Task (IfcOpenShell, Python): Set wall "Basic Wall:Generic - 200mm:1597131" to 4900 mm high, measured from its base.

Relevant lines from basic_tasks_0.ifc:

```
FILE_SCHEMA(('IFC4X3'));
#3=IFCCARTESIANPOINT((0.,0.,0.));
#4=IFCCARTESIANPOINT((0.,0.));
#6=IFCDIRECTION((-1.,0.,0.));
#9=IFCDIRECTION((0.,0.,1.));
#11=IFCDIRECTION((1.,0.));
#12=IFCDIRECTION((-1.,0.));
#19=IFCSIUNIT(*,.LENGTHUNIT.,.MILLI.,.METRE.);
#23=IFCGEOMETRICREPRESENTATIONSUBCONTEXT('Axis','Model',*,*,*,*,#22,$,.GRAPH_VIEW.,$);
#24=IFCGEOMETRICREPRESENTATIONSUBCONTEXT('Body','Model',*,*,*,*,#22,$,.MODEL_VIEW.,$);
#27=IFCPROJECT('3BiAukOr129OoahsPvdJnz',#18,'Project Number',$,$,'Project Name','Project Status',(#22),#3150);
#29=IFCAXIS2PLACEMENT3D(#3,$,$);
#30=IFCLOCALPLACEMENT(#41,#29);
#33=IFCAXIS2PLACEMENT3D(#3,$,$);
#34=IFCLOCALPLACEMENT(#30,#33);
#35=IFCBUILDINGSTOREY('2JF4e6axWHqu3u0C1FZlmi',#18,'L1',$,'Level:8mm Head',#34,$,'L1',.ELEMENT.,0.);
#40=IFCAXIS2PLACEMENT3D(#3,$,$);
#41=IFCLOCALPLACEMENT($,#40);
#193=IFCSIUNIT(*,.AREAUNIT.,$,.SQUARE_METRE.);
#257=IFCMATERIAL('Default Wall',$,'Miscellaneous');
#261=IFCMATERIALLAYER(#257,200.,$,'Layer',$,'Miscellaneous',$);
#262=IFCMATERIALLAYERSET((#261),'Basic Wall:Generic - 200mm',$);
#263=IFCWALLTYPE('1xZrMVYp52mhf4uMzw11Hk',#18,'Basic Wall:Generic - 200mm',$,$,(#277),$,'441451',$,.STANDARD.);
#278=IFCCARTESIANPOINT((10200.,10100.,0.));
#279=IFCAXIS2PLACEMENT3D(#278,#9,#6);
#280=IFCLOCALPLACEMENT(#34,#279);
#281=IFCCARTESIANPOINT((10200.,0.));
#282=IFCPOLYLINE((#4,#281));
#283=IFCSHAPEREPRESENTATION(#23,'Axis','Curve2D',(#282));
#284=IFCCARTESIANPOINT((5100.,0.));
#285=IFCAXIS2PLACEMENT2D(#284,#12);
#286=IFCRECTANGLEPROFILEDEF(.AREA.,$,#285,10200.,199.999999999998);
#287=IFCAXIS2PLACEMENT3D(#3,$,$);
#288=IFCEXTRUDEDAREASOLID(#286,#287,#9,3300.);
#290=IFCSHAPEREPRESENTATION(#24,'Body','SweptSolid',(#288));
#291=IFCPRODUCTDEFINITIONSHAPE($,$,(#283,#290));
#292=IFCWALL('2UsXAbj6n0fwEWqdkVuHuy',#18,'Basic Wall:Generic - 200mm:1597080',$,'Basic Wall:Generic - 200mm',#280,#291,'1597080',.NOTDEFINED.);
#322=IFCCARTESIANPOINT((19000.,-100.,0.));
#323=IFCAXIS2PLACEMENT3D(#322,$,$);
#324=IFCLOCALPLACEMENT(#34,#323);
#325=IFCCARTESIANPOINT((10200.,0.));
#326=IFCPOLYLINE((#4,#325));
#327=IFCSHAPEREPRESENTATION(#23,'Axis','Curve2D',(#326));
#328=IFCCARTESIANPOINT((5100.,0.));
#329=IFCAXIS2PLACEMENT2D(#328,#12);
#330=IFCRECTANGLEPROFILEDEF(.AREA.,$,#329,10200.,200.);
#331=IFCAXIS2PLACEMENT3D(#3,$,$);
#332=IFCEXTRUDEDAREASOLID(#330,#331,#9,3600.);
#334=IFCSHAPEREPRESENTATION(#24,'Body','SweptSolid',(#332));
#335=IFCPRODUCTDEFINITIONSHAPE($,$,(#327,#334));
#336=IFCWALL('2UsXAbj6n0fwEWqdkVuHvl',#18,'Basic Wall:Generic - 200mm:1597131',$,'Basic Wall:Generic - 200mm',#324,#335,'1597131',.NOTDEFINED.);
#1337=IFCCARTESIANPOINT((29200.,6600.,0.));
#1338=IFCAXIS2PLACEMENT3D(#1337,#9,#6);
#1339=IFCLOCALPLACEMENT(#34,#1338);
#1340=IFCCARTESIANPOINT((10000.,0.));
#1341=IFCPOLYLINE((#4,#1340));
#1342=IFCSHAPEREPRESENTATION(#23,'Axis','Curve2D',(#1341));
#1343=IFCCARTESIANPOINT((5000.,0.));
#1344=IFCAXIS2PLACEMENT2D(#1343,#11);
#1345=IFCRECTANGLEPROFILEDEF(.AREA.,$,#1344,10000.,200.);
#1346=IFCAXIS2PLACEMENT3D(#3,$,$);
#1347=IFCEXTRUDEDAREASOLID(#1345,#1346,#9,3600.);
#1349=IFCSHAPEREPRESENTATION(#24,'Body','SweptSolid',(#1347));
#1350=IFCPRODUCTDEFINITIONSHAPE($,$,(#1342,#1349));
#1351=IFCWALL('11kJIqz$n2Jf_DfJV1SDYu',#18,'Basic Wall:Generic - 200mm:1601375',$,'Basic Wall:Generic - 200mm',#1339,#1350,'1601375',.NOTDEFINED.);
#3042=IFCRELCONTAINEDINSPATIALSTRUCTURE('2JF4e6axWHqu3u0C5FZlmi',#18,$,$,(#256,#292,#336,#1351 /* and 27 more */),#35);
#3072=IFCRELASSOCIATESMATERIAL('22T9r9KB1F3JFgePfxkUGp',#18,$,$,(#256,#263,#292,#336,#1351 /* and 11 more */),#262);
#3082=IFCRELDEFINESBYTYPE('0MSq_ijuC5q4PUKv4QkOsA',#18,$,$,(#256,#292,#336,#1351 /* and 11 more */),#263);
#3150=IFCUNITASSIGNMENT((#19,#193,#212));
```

```python
import ifcopenshell
import ifcopenshell.geom
import ifcopenshell.util.representation
import ifcopenshell.util.shape
import ifcopenshell.util.unit

model = ifcopenshell.open("basic_tasks_0.ifc")
unit_scale = ifcopenshell.util.unit.calculate_unit_scale(model)
settings = ifcopenshell.geom.settings()


def volume(element):
    """Net volume in cubic metres, openings subtracted."""
    shape = ifcopenshell.geom.create_shape(settings, element)
    return ifcopenshell.util.shape.get_volume(shape.geometry)


wall = model.by_guid("2UsXAbj6n0fwEWqdkVuHvl")
before = volume(wall)

body = ifcopenshell.util.representation.get_representation(wall, "Model", "Body")
solid = body.Items[0]
old_height = solid.Depth
solid.Depth = 4.9 / unit_scale
after = volume(wall)

print(f"height {old_height:g} -> {solid.Depth:g}, volume {before:.3f} -> {after:.3f} m3")

model.write("basic_tasks_0_rev.ifc")
```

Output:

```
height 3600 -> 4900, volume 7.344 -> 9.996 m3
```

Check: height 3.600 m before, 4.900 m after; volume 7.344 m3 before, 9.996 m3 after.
